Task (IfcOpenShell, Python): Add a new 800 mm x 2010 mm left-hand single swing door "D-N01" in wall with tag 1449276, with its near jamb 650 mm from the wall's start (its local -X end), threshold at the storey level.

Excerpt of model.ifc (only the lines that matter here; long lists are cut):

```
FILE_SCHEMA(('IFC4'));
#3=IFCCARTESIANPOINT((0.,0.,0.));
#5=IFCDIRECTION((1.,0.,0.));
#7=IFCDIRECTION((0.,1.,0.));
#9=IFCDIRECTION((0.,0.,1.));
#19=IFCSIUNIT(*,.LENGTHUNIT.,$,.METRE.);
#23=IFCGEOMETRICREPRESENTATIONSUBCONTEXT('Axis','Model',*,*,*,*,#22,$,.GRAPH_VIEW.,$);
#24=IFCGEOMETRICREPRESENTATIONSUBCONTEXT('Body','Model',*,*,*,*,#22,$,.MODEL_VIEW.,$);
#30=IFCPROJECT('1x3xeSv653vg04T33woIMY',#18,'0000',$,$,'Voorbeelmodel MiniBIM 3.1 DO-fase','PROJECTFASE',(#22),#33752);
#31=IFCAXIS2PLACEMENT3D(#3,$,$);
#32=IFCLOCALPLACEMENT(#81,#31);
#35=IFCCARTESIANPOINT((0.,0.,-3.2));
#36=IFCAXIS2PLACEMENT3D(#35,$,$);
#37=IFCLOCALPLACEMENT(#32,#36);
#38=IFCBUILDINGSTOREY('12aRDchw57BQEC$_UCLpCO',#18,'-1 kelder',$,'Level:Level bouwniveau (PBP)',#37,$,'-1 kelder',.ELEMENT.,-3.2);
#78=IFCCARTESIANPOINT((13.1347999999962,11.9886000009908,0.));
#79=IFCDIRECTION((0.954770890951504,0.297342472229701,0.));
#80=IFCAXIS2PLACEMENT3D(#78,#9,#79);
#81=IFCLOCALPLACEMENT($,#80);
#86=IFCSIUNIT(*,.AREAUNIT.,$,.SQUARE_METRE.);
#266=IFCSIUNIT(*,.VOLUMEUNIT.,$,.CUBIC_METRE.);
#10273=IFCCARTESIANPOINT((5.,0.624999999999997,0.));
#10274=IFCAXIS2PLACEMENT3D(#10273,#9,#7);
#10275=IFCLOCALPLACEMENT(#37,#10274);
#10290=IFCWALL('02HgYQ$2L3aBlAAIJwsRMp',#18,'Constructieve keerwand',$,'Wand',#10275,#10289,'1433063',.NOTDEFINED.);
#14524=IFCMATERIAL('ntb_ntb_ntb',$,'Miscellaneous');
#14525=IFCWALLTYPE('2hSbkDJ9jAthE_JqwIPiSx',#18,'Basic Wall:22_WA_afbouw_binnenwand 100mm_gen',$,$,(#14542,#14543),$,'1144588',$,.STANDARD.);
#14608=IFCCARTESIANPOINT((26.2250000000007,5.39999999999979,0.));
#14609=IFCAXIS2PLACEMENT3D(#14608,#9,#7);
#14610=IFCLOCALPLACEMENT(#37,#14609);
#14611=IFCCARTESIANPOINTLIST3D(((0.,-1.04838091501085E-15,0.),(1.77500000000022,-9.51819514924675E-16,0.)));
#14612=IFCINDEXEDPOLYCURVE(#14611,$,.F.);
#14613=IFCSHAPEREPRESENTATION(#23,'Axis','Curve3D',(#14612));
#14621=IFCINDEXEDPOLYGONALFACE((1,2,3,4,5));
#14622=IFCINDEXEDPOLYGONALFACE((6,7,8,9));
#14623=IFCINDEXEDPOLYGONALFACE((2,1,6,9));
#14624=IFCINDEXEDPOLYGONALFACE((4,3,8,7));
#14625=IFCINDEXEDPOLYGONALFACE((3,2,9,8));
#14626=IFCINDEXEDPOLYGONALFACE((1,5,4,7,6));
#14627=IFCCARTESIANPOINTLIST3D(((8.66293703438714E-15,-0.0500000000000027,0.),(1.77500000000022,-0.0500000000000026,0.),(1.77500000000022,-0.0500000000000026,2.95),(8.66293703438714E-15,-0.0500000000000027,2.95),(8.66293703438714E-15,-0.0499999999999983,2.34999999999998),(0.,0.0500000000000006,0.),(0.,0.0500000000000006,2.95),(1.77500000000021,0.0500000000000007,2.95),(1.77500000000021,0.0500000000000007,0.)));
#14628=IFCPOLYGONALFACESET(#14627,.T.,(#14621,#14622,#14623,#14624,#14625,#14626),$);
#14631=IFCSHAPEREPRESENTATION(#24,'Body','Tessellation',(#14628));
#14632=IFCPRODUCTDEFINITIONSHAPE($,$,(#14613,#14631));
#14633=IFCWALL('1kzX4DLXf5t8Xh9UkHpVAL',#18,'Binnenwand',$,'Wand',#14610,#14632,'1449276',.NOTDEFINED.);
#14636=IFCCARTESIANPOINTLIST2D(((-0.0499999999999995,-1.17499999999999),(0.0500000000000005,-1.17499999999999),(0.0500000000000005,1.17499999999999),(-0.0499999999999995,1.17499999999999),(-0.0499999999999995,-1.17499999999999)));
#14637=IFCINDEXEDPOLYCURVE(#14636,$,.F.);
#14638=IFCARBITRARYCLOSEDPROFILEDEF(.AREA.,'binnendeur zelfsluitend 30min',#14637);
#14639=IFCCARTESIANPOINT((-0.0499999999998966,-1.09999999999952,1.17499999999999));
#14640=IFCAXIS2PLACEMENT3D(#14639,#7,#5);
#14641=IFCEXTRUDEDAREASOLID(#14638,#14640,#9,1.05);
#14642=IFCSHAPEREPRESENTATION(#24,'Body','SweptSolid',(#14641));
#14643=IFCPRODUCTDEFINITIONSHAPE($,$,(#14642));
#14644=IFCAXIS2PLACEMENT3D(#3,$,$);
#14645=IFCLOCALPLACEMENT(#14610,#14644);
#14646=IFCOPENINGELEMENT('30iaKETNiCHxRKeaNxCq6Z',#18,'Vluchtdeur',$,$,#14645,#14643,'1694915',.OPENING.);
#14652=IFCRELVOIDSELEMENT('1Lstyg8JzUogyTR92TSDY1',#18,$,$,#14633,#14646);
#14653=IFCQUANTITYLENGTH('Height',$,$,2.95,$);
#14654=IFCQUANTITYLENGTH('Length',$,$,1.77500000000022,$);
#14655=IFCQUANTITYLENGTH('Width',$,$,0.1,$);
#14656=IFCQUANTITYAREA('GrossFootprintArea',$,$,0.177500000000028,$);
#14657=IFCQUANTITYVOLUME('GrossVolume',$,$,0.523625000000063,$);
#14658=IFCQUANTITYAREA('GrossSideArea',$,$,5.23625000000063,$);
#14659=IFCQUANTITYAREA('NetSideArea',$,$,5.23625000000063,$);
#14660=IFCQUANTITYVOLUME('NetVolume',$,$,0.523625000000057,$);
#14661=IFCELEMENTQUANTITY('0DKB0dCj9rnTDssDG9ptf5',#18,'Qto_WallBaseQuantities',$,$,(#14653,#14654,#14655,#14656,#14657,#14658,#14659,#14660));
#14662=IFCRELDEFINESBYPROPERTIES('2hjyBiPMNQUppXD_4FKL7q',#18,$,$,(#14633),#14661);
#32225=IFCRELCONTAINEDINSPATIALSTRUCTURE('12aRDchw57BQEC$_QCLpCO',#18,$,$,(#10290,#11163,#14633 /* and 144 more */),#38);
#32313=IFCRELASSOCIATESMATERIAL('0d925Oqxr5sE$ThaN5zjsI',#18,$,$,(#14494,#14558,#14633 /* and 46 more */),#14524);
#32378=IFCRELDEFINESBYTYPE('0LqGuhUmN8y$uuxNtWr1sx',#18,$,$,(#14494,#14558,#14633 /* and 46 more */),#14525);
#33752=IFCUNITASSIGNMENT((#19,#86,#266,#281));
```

```python
import numpy as np
import ifcopenshell
import ifcopenshell.api.feature
import ifcopenshell.api.geometry
import ifcopenshell.api.pset
import ifcopenshell.api.root
import ifcopenshell.api.spatial
import ifcopenshell.geom
import ifcopenshell.util.element
import ifcopenshell.util.placement
import ifcopenshell.util.representation
import ifcopenshell.util.shape
import ifcopenshell.util.unit

model = ifcopenshell.open("model.ifc")
unit_scale = ifcopenshell.util.unit.calculate_unit_scale(model)
area_scale = ifcopenshell.util.unit.calculate_unit_scale(model, "AREAUNIT")
volume_scale = ifcopenshell.util.unit.calculate_unit_scale(model, "VOLUMEUNIT")
settings = ifcopenshell.geom.settings()


def volume(element):
    """Net volume in cubic metres, openings subtracted."""
    shape = ifcopenshell.geom.create_shape(settings, element)
    return ifcopenshell.util.shape.get_volume(shape.geometry)


wall = model.by_guid("1kzX4DLXf5t8Xh9UkHpVAL")
storey = ifcopenshell.util.element.get_container(wall, ifc_class="IfcBuildingStorey")
context = ifcopenshell.util.representation.get_context(model, "Model", "Body", "MODEL_VIEW")
before = volume(wall)

width, height, from_end, sill = 0.8, 2.01, 0.65, 0.0  # metres

# The wall runs along its own X axis, and the end named is its -X end.
wall_shape = ifcopenshell.geom.create_shape(settings, wall)
x, y, z = ifcopenshell.util.shape.get_vertices(wall_shape.geometry).T
start = x.min() + from_end
face, thickness = float(y.min()), float(y.max() - y.min())
wall_matrix = ifcopenshell.util.placement.get_local_placement(wall.ObjectPlacement)
level = ifcopenshell.util.placement.get_local_placement(storey.ObjectPlacement)[2, 3]


def in_wall(x, y):
    """Placement at x, y metres in the wall's axes, at sill height."""
    matrix = wall_matrix.copy()
    matrix[:, 3] = wall_matrix @ np.array([x / unit_scale, y / unit_scale, 0.0, 1.0])
    matrix[2, 3] = level + sill / unit_scale
    return matrix


# Opening: a box that overshoots both wall faces by 50 mm.
opening = ifcopenshell.api.root.create_entity(model, ifc_class="IfcOpeningElement", predefined_type="OPENING")
box = ifcopenshell.api.geometry.add_wall_representation(
    model, context=context, length=width, height=height, thickness=thickness + 0.1
)
ifcopenshell.api.geometry.assign_representation(model, product=opening, representation=box)
ifcopenshell.api.geometry.edit_object_placement(model, product=opening, matrix=in_wall(start, face - 0.05), is_si=False)
ifcopenshell.api.feature.add_feature(model, feature=opening, element=wall)

door = ifcopenshell.api.root.create_entity(model, ifc_class="IfcDoor", name="D-N01", predefined_type="DOOR")
door.OverallWidth, door.OverallHeight = width / unit_scale, height / unit_scale
door.OperationType = "SINGLE_SWING_LEFT"
body = ifcopenshell.api.geometry.add_door_representation(
    model,
    context=context,
    overall_width=door.OverallWidth,
    overall_height=door.OverallHeight,
    operation_type="SINGLE_SWING_LEFT",
    lining_properties={"LiningDepth": thickness / unit_scale, "ThresholdDepth": thickness / unit_scale},
)
ifcopenshell.api.geometry.assign_representation(model, product=door, representation=body)
ifcopenshell.api.spatial.assign_container(model, products=[door], relating_structure=storey)
ifcopenshell.api.feature.add_filling(model, opening=opening, element=door)

# The lining spans the wall, so the door starts at the wall face.
ifcopenshell.api.geometry.edit_object_placement(model, product=door, matrix=in_wall(start, face), is_si=False)

after = volume(wall)

# Update the wall's stored quantities.
qto = model.by_id(ifcopenshell.util.element.get_pset(wall, "Qto_WallBaseQuantities", should_inherit=False)["id"])
ifcopenshell.api.pset.edit_qto(model, qto=qto, properties={
    "NetSideArea": after / thickness / area_scale,
    "NetVolume": after / volume_scale,
})

print(f"wall volume {before:.3f} -> {after:.3f} m3")

model.write("model_updated.ifc")
```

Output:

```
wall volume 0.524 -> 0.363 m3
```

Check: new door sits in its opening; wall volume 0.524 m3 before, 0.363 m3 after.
